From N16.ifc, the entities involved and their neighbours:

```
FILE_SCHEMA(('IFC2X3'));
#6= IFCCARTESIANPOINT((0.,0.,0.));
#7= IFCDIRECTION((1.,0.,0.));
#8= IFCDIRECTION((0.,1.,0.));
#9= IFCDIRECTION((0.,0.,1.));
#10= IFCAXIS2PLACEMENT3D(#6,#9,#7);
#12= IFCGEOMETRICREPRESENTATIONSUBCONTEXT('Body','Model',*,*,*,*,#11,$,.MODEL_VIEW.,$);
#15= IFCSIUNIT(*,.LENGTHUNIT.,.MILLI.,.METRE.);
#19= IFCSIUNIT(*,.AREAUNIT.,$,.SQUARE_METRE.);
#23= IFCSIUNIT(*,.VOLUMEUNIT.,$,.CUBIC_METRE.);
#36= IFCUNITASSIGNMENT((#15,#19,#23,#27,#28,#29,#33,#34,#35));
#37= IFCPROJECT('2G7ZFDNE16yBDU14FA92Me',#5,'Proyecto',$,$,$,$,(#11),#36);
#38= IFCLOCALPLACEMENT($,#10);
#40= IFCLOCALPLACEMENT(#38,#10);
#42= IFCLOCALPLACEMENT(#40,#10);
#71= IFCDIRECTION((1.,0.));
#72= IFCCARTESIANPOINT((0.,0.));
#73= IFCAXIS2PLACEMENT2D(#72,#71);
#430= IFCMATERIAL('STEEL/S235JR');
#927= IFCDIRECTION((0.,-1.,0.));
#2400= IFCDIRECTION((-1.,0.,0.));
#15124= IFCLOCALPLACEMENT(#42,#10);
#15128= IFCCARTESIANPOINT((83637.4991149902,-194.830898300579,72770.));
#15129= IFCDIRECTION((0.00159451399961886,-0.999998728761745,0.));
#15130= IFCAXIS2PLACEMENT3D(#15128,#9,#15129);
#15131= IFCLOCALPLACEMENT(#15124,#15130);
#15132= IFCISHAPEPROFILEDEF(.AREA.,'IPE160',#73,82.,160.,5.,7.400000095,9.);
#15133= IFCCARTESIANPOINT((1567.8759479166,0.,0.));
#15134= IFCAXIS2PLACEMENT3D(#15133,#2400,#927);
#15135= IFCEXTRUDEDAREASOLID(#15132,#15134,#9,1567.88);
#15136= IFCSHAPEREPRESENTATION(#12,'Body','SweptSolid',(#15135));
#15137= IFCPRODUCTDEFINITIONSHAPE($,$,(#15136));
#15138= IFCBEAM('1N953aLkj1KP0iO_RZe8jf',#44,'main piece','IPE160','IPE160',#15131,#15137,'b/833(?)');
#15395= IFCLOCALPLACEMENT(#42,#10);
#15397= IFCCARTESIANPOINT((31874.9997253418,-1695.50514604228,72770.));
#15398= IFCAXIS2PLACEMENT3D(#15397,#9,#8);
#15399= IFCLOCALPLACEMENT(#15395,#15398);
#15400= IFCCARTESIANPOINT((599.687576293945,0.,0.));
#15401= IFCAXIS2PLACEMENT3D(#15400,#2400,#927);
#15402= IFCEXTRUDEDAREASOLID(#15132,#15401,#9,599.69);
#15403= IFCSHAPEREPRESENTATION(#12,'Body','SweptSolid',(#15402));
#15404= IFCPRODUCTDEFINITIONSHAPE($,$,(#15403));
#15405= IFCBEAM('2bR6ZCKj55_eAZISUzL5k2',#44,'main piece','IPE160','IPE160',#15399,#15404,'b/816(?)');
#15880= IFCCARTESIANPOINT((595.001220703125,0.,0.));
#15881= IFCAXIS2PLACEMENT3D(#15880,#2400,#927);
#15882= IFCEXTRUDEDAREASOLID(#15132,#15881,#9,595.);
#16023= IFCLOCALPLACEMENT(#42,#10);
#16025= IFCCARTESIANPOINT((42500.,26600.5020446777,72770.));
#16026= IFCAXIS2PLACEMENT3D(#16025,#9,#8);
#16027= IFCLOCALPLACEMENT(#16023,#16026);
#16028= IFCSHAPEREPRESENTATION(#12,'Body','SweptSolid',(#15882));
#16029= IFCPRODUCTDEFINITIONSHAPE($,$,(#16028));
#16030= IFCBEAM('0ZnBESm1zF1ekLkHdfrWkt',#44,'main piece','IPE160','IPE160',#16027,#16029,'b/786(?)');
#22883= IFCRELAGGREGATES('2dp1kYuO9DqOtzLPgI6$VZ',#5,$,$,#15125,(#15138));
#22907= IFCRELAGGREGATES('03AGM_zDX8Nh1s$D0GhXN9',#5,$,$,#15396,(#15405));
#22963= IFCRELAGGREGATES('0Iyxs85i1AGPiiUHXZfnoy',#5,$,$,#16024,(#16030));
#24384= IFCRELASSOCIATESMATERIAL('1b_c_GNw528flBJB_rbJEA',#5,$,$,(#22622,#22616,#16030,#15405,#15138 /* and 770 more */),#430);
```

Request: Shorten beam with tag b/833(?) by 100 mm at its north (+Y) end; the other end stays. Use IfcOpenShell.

```python
import ifcopenshell
import ifcopenshell.util.representation

model = ifcopenshell.open("N16.ifc")

member = model.by_guid("1N953aLkj1KP0iO_RZe8jf")
change = -100.0

# The extrusion runs towards the end named, so only its depth changes.
body = ifcopenshell.util.representation.get_representation(member, "Model", "Body")
solid = body.Items[0]
old_length = solid.Depth
solid.Depth += change

print(f"length {old_length:g} -> {solid.Depth:g}")

model.write("N16_rev.ifc")
```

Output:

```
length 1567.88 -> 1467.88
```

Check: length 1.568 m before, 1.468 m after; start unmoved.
